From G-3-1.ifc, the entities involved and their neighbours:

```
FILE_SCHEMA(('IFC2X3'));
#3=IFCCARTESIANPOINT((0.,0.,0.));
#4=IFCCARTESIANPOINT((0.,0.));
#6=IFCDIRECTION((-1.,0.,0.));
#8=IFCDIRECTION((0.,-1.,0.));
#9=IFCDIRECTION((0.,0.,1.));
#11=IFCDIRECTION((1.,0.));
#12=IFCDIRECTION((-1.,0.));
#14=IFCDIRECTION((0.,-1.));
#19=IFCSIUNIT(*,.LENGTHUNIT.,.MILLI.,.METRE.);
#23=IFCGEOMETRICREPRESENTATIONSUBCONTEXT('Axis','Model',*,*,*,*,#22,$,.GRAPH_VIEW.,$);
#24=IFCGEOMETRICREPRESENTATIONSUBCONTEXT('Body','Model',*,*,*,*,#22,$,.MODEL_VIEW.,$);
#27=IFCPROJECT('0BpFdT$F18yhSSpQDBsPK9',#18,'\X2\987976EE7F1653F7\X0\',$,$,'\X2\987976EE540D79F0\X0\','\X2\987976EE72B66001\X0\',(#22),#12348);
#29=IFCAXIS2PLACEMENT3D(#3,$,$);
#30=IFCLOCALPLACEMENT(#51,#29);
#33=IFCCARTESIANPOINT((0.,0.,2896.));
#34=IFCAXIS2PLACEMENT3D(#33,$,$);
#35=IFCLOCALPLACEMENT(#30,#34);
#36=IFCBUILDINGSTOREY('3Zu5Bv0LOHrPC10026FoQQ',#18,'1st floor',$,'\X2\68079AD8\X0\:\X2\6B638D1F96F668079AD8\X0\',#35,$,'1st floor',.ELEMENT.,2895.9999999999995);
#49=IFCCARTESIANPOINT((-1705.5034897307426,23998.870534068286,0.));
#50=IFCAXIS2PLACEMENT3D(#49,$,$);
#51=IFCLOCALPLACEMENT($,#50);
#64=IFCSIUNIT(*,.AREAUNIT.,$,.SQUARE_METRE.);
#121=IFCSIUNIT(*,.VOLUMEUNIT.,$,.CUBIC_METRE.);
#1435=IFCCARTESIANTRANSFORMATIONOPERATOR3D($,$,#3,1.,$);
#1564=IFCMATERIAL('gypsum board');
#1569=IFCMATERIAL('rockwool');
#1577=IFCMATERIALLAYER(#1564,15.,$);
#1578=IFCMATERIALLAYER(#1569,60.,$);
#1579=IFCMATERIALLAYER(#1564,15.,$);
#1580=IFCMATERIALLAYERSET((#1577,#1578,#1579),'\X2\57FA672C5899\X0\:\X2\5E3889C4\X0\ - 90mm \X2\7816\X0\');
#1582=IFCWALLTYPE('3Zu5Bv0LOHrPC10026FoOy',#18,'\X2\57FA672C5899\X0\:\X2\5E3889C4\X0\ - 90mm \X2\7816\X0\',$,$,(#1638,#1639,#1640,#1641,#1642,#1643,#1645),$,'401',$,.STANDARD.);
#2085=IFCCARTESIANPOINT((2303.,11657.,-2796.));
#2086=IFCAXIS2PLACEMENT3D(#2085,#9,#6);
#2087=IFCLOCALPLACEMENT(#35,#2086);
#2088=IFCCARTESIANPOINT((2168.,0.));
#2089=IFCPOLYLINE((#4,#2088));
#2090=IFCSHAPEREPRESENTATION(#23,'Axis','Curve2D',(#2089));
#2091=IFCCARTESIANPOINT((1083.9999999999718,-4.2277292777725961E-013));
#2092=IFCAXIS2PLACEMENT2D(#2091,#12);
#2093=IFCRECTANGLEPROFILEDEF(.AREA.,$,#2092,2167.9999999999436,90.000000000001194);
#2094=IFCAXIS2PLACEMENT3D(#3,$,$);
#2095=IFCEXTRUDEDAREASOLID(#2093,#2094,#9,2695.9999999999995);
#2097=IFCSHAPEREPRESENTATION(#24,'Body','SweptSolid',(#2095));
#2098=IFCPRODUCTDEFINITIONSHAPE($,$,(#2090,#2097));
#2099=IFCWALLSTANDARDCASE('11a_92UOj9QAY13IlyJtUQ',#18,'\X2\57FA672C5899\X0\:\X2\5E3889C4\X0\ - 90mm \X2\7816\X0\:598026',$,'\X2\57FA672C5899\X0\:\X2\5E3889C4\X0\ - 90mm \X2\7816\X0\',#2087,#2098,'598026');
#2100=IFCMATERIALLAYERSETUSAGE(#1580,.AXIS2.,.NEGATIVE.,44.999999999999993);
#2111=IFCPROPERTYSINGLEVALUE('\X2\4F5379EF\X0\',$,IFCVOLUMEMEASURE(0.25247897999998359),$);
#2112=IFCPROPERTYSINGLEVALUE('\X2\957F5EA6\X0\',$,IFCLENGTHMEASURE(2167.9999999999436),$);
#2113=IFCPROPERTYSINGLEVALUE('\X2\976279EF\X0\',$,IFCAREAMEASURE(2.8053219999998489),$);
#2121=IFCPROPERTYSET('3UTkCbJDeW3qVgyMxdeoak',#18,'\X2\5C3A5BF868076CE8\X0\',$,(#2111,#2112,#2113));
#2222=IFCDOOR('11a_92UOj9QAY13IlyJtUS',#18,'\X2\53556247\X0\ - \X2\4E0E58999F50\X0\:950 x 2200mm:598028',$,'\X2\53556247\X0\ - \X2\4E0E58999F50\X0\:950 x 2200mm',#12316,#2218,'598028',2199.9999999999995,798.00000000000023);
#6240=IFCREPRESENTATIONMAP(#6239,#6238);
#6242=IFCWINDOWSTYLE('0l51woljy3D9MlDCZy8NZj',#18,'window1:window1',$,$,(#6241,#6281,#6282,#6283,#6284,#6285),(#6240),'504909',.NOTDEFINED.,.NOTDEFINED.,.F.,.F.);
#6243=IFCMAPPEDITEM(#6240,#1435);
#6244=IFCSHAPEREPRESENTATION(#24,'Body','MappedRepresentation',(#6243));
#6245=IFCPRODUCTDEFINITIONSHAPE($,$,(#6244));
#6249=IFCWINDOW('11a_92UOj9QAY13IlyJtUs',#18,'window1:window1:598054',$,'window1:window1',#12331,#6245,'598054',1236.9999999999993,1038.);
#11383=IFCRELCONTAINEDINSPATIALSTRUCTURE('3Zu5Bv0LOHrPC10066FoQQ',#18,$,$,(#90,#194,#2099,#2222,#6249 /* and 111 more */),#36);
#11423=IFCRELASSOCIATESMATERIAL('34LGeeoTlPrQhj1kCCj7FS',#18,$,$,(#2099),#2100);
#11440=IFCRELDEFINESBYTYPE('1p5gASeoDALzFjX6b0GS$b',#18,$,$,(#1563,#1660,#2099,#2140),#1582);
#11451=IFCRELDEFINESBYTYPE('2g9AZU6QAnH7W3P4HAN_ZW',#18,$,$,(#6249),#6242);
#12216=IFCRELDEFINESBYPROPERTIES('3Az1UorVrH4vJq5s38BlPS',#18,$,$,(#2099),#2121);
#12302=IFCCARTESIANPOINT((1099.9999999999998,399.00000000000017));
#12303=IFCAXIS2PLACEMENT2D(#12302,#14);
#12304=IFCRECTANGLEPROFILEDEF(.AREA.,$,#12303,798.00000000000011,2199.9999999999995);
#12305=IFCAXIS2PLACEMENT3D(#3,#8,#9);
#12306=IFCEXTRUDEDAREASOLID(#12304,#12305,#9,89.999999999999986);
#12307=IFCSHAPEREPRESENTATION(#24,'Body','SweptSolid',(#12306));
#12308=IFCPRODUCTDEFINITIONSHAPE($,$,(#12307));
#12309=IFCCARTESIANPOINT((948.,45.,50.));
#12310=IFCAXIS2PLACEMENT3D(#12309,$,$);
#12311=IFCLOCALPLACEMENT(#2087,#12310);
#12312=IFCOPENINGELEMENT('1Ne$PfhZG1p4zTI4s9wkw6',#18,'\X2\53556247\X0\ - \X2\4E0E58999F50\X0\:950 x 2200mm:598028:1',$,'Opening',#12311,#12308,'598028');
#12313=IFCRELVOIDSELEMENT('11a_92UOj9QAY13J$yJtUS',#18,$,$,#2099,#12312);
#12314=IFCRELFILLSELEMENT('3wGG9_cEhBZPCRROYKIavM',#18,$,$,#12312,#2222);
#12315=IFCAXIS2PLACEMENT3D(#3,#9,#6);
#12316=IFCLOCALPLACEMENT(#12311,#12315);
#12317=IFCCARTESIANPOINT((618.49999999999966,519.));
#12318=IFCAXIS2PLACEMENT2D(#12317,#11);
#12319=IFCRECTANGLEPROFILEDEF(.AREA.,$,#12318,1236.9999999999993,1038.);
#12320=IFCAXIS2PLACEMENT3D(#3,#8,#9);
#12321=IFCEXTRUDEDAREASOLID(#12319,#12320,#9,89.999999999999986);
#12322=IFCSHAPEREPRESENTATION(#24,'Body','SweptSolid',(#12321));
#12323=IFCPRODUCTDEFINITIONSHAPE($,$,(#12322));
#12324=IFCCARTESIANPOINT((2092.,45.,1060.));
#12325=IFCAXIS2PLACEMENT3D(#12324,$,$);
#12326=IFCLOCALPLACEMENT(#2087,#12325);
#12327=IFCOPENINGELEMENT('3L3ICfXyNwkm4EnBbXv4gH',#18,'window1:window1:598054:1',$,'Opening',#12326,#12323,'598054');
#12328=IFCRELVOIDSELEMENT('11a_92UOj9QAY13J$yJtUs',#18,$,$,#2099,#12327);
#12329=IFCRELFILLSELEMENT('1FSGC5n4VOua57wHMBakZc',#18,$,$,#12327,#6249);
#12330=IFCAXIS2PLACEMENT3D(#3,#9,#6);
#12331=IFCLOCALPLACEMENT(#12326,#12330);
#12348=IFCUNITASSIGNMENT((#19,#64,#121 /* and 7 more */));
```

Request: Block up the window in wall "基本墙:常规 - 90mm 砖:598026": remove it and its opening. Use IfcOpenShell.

```python
import ifcopenshell
import ifcopenshell.api.feature
import ifcopenshell.api.pset
import ifcopenshell.api.root
import ifcopenshell.geom
import ifcopenshell.util.element
import ifcopenshell.util.shape
import ifcopenshell.util.unit

model = ifcopenshell.open("G-3-1.ifc")
area_scale = ifcopenshell.util.unit.calculate_unit_scale(model, "AREAUNIT")
volume_scale = ifcopenshell.util.unit.calculate_unit_scale(model, "VOLUMEUNIT")
settings = ifcopenshell.geom.settings()


def volume(element):
    """Net volume in cubic metres, openings subtracted."""
    shape = ifcopenshell.geom.create_shape(settings, element)
    return ifcopenshell.util.shape.get_volume(shape.geometry)


window = model.by_id(6249)
opening = window.FillsVoids[0].RelatingOpeningElement
wall = opening.VoidsElements[0].RelatingBuildingElement
before = volume(wall)

ifcopenshell.api.root.remove_product(model, product=window)
ifcopenshell.api.feature.remove_feature(model, feature=opening)

after = volume(wall)
thickness = 0.09  # wall thickness in metres

# Update the wall's stored quantities.
pset = model.by_id(ifcopenshell.util.element.get_pset(wall, "尺寸标注", should_inherit=False)["id"])
ifcopenshell.api.pset.edit_pset(model, pset=pset, properties={
    "体积": model.create_entity("IfcVolumeMeasure", after / volume_scale),
    "面积": model.create_entity("IfcAreaMeasure", after / thickness / area_scale),
})

print(f"wall volume {before:.3f} -> {after:.3f} m3")

model.write("G-3-1_v2.ifc")
```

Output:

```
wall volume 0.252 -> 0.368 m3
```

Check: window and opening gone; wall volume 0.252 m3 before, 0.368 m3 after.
